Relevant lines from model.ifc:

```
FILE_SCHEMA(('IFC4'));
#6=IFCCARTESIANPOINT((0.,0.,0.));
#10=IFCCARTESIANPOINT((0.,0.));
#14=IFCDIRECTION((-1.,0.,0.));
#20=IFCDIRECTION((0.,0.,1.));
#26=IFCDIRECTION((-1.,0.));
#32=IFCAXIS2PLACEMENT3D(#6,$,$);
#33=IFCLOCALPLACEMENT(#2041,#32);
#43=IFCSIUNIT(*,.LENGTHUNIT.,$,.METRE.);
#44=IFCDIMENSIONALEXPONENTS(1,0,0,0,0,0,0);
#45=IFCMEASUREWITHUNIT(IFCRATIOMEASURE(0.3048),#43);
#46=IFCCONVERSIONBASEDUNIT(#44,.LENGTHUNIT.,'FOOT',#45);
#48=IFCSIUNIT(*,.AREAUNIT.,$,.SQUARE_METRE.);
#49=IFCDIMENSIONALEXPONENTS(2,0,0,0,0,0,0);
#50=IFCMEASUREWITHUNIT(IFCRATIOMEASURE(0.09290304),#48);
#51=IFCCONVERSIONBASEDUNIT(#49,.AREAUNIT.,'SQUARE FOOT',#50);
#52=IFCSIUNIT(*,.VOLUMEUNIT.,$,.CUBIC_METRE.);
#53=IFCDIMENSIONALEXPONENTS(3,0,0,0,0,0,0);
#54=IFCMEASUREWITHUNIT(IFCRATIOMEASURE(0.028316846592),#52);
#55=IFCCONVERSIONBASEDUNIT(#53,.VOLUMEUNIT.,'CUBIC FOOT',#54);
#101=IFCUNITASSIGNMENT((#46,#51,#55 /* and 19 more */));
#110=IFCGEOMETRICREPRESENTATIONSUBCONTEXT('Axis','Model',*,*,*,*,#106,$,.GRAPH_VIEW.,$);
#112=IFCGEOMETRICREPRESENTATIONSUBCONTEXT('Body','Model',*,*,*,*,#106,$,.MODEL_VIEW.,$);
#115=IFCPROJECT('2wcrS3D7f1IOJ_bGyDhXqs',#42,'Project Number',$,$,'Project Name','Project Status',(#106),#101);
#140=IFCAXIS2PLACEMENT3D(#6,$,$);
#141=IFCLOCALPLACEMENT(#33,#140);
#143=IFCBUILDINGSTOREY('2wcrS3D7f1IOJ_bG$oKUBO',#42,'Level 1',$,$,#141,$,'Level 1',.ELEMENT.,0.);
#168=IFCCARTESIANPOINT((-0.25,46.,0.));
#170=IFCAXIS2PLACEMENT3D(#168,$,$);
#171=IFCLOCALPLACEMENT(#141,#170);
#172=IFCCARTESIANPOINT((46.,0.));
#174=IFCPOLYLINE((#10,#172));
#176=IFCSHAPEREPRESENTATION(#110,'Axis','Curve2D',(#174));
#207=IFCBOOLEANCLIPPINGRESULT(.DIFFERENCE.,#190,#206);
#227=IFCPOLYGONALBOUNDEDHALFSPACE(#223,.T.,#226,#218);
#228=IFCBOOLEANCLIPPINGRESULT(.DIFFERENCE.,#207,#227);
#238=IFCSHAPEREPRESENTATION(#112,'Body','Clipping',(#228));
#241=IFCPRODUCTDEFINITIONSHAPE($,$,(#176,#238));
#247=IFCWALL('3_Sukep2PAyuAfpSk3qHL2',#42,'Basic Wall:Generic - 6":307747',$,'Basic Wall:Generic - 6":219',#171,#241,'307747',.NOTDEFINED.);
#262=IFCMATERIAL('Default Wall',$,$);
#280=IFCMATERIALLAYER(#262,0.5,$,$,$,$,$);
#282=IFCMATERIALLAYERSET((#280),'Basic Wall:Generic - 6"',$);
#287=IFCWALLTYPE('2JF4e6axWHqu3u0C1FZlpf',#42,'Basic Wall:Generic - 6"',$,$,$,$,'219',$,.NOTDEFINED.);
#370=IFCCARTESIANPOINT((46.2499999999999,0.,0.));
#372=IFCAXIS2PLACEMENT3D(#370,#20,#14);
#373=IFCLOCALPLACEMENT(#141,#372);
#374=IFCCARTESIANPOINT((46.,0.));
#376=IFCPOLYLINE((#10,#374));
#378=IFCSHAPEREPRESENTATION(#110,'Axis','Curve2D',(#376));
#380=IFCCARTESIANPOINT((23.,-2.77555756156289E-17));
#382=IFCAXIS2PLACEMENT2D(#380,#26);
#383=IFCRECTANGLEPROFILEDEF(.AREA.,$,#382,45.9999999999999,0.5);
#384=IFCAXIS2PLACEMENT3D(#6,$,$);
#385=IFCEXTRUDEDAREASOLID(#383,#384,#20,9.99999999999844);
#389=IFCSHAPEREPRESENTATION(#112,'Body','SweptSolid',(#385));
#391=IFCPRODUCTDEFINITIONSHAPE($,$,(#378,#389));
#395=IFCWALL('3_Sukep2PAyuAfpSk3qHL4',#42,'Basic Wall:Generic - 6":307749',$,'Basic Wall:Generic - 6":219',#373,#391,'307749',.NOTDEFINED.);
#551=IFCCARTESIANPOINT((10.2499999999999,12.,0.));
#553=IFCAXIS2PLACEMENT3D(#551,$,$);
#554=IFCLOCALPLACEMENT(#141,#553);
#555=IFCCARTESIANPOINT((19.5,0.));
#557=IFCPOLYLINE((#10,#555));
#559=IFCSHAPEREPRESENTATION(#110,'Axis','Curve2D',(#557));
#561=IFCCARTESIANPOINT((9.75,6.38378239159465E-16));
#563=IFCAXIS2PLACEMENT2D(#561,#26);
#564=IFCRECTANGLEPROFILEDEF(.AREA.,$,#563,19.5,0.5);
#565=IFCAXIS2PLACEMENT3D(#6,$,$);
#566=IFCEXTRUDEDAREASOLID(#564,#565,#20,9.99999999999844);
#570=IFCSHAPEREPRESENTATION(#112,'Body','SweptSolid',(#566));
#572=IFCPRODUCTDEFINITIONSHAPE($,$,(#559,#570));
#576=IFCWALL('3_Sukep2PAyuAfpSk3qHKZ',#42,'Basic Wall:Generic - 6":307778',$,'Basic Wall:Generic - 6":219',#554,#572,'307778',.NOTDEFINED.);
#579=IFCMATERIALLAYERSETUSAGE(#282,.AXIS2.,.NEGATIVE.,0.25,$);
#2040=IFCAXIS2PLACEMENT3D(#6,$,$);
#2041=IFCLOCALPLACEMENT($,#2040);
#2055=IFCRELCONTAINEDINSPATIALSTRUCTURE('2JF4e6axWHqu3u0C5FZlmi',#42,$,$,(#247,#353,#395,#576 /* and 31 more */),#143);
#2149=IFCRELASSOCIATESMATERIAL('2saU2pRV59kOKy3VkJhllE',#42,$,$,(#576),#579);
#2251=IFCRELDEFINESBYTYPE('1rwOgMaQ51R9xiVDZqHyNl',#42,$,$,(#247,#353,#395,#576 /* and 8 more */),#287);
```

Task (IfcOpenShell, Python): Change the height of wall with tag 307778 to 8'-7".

```python
import ifcopenshell
import ifcopenshell.geom
import ifcopenshell.util.representation
import ifcopenshell.util.shape
import ifcopenshell.util.unit

model = ifcopenshell.open("model.ifc")
unit_scale = ifcopenshell.util.unit.calculate_unit_scale(model)
settings = ifcopenshell.geom.settings()


def volume(element):
    """Net volume in cubic metres, openings subtracted."""
    shape = ifcopenshell.geom.create_shape(settings, element)
    return ifcopenshell.util.shape.get_volume(shape.geometry)


wall = model.by_id(576)
before = volume(wall)

body = ifcopenshell.util.representation.get_representation(wall, "Model", "Body")
solid = body.Items[0]
old_height = solid.Depth
solid.Depth = 103 * 0.0254 / unit_scale
after = volume(wall)

print(f"height {old_height:g} -> {solid.Depth:g}, volume {before:.3f} -> {after:.3f} m3")

model.write("model_v2.ifc")
```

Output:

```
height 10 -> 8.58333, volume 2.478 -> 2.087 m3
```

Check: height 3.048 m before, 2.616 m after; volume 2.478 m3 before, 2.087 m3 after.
